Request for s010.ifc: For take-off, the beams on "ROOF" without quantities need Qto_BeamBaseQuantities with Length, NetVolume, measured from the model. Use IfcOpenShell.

First a look at what the model holds.

```python
import ifcopenshell
import ifcopenshell.util.element
import ifcopenshell.util.unit

model = ifcopenshell.open("s010.ifc")
print(model.schema)
for unit_type in ("LENGTHUNIT", "AREAUNIT", "VOLUMEUNIT"):
    print(unit_type, ifcopenshell.util.unit.calculate_unit_scale(model, unit_type))
storey = next(s for s in model.by_type("IfcBuildingStorey") if s.Name == "ROOF")
beams = [e for e in ifcopenshell.util.element.get_decomposition(storey) if e.is_a("IfcBeam")]
for e in sorted(beams, key=lambda e: e.id()):
    print(e.id(), e.is_a(), e.Name, list(ifcopenshell.util.element.get_psets(e, qtos_only=True)), sep=" | ")
```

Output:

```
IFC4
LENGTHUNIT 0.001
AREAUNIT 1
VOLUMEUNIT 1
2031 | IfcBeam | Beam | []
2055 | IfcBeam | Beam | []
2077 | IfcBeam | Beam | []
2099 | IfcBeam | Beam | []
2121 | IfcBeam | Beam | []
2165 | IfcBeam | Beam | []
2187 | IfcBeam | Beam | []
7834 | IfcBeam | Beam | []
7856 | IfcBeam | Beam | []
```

```python
import ifcopenshell
import ifcopenshell.api.pset
import ifcopenshell.geom
import ifcopenshell.util.element
import ifcopenshell.util.shape
import ifcopenshell.util.unit

model = ifcopenshell.open("s010.ifc")
unit_scale = ifcopenshell.util.unit.calculate_unit_scale(model)
volume_scale = ifcopenshell.util.unit.calculate_unit_scale(model, "VOLUMEUNIT")
settings = ifcopenshell.geom.settings()

storey = next(s for s in model.by_type("IfcBuildingStorey") if s.Name == "ROOF")
beams = [e for e in ifcopenshell.util.element.get_decomposition(storey) if e.is_a("IfcBeam")]

for e in sorted(beams, key=lambda e: e.id()):
    if ifcopenshell.util.element.get_psets(e, qtos_only=True, should_inherit=False):
        continue
    # Geometry comes back in metres, in the element's own axes.
    shape = ifcopenshell.geom.create_shape(settings, e)
    values = {
        "Length": ifcopenshell.util.shape.get_max_xyz(shape.geometry) / unit_scale,
        "NetVolume": ifcopenshell.util.shape.get_volume(shape.geometry) / volume_scale,
    }
    qto = ifcopenshell.api.pset.add_qto(model, product=e, name="Qto_BeamBaseQuantities")
    ifcopenshell.api.pset.edit_qto(model, qto=qto, properties=values)
    print(e.id(), {k: round(v, 3) for k, v in values.items()})

model.write("s010_updated.ifc")
```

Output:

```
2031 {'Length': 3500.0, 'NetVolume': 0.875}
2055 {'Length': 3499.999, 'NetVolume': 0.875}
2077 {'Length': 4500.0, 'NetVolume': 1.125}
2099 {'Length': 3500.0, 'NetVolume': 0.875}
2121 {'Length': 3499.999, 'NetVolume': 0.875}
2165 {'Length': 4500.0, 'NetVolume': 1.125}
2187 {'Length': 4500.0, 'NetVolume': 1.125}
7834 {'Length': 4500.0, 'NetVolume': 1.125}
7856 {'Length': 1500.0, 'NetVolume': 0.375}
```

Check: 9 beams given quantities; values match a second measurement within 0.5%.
